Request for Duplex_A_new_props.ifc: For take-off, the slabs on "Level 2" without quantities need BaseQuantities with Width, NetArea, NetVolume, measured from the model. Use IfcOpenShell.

First a look at what the model holds.

```python
import ifcopenshell
import ifcopenshell.util.element
import ifcopenshell.util.unit

model = ifcopenshell.open("Duplex_A_new_props.ifc")
print(model.schema)
for unit_type in ("LENGTHUNIT", "AREAUNIT", "VOLUMEUNIT"):
    print(unit_type, ifcopenshell.util.unit.calculate_unit_scale(model, unit_type))
storey = next(s for s in model.by_type("IfcBuildingStorey") if s.Name == "Level 2")
slabs = [e for e in ifcopenshell.util.element.get_decomposition(storey) if e.is_a("IfcSlab")]
for e in sorted(slabs, key=lambda e: e.id()):
    print(e.id(), e.is_a(), e.Name, list(ifcopenshell.util.element.get_psets(e, qtos_only=True)), sep=" | ")
```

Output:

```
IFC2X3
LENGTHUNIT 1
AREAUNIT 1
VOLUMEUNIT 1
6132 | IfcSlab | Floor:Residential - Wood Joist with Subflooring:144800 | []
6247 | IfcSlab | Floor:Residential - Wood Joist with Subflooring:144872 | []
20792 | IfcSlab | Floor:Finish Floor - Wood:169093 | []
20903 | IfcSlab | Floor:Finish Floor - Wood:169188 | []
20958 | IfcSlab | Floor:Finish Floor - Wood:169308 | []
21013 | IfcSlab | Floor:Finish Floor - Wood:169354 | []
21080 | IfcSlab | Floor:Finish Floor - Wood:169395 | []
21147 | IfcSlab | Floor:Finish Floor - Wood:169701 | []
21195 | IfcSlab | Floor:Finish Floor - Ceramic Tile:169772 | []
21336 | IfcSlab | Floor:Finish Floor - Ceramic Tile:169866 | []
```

```python
import ifcopenshell
import ifcopenshell.api.pset
import ifcopenshell.geom
import ifcopenshell.util.element
import ifcopenshell.util.shape
import ifcopenshell.util.unit

model = ifcopenshell.open("Duplex_A_new_props.ifc")
unit_scale = ifcopenshell.util.unit.calculate_unit_scale(model)
area_scale = ifcopenshell.util.unit.calculate_unit_scale(model, "AREAUNIT")
volume_scale = ifcopenshell.util.unit.calculate_unit_scale(model, "VOLUMEUNIT")
settings = ifcopenshell.geom.settings()

storey = next(s for s in model.by_type("IfcBuildingStorey") if s.Name == "Level 2")
slabs = [e for e in ifcopenshell.util.element.get_decomposition(storey) if e.is_a("IfcSlab")]

for e in sorted(slabs, key=lambda e: e.id()):
    if ifcopenshell.util.element.get_psets(e, qtos_only=True, should_inherit=False):
        continue
    # Geometry comes back in metres, in the element's own axes.
    shape = ifcopenshell.geom.create_shape(settings, e)
    values = {
        "Width": ifcopenshell.util.shape.get_z(shape.geometry) / unit_scale,
        "NetArea": ifcopenshell.util.shape.get_footprint_area(shape.geometry) / area_scale,
        "NetVolume": ifcopenshell.util.shape.get_volume(shape.geometry) / volume_scale,
    }
    qto = ifcopenshell.api.pset.add_qto(model, product=e, name="BaseQuantities")
    ifcopenshell.api.pset.edit_qto(model, qto=qto, properties=values)
    print(e.id(), {k: round(v, 3) for k, v in values.items()})

model.write("Duplex_A_new_props_rev.ifc")
```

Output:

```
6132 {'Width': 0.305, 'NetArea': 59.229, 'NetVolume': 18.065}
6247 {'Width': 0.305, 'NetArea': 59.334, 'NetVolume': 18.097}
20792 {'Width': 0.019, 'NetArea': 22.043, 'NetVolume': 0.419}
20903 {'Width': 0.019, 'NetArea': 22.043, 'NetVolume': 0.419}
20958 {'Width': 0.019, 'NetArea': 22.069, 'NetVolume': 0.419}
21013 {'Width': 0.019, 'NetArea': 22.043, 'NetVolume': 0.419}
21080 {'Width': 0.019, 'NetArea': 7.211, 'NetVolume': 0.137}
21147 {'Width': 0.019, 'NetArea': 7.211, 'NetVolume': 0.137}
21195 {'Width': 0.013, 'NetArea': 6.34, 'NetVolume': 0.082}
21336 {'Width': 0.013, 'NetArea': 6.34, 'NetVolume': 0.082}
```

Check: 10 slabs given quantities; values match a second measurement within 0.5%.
